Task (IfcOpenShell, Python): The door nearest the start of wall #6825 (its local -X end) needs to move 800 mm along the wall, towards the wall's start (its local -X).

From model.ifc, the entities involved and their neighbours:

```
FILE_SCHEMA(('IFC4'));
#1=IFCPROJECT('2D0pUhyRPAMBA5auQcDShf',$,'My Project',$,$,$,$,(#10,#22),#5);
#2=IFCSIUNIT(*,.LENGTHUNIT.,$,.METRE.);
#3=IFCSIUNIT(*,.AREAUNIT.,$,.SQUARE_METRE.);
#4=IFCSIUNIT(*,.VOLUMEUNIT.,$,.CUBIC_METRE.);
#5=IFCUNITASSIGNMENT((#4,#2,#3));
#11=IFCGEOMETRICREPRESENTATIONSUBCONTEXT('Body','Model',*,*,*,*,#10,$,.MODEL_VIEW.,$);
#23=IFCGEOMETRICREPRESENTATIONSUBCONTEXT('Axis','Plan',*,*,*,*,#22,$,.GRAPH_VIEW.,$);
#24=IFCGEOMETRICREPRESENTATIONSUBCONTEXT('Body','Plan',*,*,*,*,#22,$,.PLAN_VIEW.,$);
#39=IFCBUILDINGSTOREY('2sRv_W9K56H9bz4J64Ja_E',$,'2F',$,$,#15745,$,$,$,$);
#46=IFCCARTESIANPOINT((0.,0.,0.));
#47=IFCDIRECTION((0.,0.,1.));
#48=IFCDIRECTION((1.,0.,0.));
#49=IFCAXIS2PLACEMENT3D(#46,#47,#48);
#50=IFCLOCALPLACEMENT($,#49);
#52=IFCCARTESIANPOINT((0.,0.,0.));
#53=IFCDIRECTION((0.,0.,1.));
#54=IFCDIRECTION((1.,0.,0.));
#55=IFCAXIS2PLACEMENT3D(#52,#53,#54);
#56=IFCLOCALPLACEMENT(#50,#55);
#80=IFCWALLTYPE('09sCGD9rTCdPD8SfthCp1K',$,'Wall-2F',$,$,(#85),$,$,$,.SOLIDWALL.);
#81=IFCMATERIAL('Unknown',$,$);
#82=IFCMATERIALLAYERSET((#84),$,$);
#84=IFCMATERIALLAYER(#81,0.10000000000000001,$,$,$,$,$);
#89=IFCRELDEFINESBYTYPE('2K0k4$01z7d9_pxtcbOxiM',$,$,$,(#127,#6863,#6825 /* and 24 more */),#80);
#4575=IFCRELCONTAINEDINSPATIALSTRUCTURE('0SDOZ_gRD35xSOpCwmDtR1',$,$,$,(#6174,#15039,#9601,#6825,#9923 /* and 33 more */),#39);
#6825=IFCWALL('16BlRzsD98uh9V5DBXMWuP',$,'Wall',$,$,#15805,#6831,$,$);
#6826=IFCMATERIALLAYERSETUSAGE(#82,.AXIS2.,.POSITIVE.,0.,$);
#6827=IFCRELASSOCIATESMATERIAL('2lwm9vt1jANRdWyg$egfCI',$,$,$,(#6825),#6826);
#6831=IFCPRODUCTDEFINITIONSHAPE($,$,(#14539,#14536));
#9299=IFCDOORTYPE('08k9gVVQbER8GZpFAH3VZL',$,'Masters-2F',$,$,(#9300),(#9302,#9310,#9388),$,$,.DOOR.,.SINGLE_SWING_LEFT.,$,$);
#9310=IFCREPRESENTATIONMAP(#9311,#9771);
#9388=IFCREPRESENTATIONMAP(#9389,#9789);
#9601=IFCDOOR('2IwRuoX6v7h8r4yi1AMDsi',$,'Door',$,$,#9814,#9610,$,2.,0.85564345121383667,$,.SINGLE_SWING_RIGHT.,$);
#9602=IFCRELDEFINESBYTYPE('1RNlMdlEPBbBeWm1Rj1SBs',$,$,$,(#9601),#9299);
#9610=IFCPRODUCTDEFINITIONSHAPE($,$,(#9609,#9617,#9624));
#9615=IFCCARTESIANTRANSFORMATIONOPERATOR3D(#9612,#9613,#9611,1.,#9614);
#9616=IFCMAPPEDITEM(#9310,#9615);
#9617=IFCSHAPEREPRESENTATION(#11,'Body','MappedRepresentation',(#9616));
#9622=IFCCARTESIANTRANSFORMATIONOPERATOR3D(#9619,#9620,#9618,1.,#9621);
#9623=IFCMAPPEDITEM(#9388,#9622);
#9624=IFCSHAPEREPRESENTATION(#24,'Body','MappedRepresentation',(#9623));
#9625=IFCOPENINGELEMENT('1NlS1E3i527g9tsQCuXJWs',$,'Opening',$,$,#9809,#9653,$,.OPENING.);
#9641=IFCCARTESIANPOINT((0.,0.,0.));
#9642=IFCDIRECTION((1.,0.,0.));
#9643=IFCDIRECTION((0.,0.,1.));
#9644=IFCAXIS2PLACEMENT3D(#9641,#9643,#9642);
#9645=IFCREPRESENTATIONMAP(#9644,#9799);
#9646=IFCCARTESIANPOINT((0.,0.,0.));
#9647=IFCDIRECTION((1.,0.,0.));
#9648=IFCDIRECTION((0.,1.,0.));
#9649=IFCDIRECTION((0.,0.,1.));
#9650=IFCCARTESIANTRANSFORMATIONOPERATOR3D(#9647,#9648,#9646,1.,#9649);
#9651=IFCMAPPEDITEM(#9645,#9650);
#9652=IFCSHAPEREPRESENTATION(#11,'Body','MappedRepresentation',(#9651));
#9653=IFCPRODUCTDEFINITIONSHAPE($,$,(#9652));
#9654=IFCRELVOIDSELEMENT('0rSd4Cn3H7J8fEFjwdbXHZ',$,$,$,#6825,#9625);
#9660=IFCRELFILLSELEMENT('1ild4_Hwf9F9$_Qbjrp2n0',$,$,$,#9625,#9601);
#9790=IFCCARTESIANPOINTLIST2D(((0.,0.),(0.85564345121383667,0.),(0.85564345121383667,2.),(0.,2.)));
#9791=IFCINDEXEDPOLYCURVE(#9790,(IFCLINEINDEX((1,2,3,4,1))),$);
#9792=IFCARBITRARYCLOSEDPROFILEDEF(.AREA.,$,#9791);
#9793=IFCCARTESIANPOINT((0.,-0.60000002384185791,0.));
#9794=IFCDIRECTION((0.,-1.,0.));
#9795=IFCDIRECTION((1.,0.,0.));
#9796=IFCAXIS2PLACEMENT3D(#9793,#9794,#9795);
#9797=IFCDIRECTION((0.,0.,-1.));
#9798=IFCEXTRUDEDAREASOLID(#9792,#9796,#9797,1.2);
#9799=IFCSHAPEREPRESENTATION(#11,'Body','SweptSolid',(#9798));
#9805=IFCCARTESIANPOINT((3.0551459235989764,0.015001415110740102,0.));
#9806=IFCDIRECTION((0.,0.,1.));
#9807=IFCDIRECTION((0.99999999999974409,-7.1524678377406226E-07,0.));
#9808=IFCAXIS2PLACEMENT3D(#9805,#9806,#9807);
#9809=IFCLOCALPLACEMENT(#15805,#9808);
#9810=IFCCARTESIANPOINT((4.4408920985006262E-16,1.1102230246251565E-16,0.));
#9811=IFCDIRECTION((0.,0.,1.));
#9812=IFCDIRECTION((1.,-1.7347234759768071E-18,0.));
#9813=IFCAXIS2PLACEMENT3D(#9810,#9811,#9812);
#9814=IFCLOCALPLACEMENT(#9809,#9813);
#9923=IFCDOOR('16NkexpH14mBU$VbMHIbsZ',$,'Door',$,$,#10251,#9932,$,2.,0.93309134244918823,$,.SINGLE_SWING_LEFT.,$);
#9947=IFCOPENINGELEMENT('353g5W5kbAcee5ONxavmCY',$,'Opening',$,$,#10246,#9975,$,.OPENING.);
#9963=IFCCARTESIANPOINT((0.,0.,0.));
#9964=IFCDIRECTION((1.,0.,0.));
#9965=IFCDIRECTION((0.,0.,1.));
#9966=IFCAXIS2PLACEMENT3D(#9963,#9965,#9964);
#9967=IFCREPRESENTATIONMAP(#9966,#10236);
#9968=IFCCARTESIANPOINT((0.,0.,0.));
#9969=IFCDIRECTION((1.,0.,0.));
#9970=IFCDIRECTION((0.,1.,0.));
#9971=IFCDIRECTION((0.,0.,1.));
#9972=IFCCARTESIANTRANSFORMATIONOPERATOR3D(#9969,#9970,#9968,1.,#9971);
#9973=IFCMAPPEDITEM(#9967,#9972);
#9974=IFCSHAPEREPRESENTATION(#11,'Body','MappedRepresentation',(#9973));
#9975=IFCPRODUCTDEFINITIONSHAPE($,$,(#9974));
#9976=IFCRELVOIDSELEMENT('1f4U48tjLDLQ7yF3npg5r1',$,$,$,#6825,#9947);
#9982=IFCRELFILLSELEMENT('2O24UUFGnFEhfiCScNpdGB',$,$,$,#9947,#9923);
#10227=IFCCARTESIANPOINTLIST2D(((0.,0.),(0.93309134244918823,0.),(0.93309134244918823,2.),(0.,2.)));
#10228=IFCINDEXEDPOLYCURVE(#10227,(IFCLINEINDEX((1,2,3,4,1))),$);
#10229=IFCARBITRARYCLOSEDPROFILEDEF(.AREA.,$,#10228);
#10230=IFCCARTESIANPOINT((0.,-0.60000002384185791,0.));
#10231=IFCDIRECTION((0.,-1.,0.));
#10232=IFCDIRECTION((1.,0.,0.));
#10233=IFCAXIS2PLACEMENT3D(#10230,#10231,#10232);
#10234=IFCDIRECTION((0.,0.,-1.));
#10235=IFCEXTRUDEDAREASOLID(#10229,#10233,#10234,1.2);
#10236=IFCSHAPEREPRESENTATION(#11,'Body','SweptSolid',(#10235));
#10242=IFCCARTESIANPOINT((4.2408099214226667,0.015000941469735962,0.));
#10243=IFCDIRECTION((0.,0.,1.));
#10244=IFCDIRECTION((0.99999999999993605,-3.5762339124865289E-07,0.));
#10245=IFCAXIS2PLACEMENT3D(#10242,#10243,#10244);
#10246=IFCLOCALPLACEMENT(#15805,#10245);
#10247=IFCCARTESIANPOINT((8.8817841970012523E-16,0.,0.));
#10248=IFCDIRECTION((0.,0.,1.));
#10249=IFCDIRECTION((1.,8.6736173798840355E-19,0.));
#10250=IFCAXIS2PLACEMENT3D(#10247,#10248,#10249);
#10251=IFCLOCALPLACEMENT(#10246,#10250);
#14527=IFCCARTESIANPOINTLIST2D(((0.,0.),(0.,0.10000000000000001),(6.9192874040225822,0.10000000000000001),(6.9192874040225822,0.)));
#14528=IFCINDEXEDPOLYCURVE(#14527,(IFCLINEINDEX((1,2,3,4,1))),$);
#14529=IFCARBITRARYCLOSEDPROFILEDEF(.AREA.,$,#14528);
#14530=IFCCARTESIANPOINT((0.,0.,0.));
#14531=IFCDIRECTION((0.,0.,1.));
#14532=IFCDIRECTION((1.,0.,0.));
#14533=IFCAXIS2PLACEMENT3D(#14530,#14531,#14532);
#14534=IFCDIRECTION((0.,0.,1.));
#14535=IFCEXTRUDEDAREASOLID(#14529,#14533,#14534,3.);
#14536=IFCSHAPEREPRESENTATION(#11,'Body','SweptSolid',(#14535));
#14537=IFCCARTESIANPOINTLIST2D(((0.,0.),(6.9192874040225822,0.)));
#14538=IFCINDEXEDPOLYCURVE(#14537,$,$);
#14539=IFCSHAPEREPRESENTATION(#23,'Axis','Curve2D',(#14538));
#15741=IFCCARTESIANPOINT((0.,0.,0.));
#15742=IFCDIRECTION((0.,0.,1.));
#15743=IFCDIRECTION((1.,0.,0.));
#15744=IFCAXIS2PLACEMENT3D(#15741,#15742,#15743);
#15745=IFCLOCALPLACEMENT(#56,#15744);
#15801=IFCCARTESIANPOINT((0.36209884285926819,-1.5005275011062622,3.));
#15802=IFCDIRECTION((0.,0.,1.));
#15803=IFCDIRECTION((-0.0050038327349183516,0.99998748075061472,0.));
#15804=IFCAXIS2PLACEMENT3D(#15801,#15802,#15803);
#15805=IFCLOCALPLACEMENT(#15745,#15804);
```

```python
import ifcopenshell
import ifcopenshell.api.geometry
import ifcopenshell.util.placement
import ifcopenshell.util.unit

model = ifcopenshell.open("model.ifc")
unit_scale = ifcopenshell.util.unit.calculate_unit_scale(model)

door = model.by_guid("2IwRuoX6v7h8r4yi1AMDsi")
opening = door.FillsVoids[0].RelatingOpeningElement
wall = opening.VoidsElements[0].RelatingBuildingElement

wall_matrix = ifcopenshell.util.placement.get_local_placement(wall.ObjectPlacement)
shift = wall_matrix[:3, 0] * -0.8 / unit_scale
before = ifcopenshell.util.placement.get_local_placement(door.ObjectPlacement)[:3, 3].copy()

# The door is placed relative to its opening, so it follows when the opening moves.
matrix = ifcopenshell.util.placement.get_local_placement(opening.ObjectPlacement)
matrix[:3, 3] += shift
ifcopenshell.api.geometry.edit_object_placement(
    model, product=opening, matrix=matrix, is_si=False, should_transform_children=True
)

after = ifcopenshell.util.placement.get_local_placement(door.ObjectPlacement)[:3, 3]
print("door moved by", (after - before).round(3) + 0.0)

model.write("model-out.ifc")
```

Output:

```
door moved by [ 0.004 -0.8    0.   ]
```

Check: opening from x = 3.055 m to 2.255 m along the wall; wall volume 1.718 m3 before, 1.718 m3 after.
